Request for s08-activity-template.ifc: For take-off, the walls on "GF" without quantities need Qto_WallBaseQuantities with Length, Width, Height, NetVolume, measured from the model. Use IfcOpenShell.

First a look at what the model holds.

```python
import ifcopenshell
import ifcopenshell.util.element
import ifcopenshell.util.unit

model = ifcopenshell.open("s08-activity-template.ifc")
print(model.schema)
for unit_type in ("LENGTHUNIT", "AREAUNIT", "VOLUMEUNIT"):
    print(unit_type, ifcopenshell.util.unit.calculate_unit_scale(model, unit_type))
storey = next(s for s in model.by_type("IfcBuildingStorey") if s.Name == "GF")
walls = [e for e in ifcopenshell.util.element.get_decomposition(storey) if e.is_a("IfcWall")]
for e in sorted(walls, key=lambda e: e.id()):
    print(e.id(), e.is_a(), e.Name, list(ifcopenshell.util.element.get_psets(e, qtos_only=True)), sep=" | ")
```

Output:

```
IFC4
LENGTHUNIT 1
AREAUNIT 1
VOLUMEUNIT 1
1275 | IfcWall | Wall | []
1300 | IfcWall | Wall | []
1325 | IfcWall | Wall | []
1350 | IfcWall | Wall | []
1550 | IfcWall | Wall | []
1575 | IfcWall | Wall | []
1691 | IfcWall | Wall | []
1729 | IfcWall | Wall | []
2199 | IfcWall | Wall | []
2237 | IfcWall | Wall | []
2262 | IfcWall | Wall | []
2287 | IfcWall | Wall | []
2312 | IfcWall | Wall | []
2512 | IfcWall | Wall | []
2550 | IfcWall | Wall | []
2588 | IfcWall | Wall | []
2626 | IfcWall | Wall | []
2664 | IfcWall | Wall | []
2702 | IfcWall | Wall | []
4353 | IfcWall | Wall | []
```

```python
import ifcopenshell
import ifcopenshell.api.pset
import ifcopenshell.geom
import ifcopenshell.util.element
import ifcopenshell.util.shape
import ifcopenshell.util.unit

model = ifcopenshell.open("s08-activity-template.ifc")
unit_scale = ifcopenshell.util.unit.calculate_unit_scale(model)
volume_scale = ifcopenshell.util.unit.calculate_unit_scale(model, "VOLUMEUNIT")
settings = ifcopenshell.geom.settings()

storey = next(s for s in model.by_type("IfcBuildingStorey") if s.Name == "GF")
walls = [e for e in ifcopenshell.util.element.get_decomposition(storey) if e.is_a("IfcWall")]

for e in sorted(walls, key=lambda e: e.id()):
    if ifcopenshell.util.element.get_psets(e, qtos_only=True, should_inherit=False):
        continue
    # Geometry comes back in metres, in the element's own axes.
    shape = ifcopenshell.geom.create_shape(settings, e)
    values = {
        "Length": ifcopenshell.util.shape.get_x(shape.geometry) / unit_scale,
        "Width": ifcopenshell.util.shape.get_y(shape.geometry) / unit_scale,
        "Height": ifcopenshell.util.shape.get_z(shape.geometry) / unit_scale,
        "NetVolume": ifcopenshell.util.shape.get_volume(shape.geometry) / volume_scale,
    }
    qto = ifcopenshell.api.pset.add_qto(model, product=e, name="Qto_WallBaseQuantities")
    ifcopenshell.api.pset.edit_qto(model, qto=qto, properties=values)
    print(e.id(), {k: round(v, 3) for k, v in values.items()})

model.write("s08-activity-template_updated.ifc")
```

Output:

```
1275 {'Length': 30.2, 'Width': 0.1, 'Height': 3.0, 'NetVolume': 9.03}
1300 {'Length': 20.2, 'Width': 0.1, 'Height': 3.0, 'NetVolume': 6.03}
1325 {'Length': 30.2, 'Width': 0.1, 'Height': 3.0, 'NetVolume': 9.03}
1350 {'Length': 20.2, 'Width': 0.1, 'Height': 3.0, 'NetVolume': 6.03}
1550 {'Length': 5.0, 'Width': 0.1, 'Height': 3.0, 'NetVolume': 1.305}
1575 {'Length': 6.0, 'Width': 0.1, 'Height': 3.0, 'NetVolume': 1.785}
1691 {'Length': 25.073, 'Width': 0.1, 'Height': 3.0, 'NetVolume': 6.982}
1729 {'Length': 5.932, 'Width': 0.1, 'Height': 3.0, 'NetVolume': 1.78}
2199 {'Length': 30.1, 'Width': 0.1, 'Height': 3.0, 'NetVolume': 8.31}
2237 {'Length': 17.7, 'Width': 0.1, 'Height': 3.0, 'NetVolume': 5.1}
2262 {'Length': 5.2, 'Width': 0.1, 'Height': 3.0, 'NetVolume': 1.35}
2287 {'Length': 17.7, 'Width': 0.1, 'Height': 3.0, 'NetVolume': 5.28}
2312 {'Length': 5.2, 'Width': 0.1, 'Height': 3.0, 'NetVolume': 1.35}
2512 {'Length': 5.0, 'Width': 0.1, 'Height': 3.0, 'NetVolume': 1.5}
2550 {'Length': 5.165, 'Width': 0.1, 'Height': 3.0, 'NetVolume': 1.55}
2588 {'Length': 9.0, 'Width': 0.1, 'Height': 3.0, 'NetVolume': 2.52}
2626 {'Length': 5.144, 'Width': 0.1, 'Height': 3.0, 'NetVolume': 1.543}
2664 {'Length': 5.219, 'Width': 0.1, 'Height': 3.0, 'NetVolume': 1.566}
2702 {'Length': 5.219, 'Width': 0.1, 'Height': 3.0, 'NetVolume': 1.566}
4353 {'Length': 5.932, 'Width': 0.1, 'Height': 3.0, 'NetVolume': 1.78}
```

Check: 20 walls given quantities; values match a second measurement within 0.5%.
